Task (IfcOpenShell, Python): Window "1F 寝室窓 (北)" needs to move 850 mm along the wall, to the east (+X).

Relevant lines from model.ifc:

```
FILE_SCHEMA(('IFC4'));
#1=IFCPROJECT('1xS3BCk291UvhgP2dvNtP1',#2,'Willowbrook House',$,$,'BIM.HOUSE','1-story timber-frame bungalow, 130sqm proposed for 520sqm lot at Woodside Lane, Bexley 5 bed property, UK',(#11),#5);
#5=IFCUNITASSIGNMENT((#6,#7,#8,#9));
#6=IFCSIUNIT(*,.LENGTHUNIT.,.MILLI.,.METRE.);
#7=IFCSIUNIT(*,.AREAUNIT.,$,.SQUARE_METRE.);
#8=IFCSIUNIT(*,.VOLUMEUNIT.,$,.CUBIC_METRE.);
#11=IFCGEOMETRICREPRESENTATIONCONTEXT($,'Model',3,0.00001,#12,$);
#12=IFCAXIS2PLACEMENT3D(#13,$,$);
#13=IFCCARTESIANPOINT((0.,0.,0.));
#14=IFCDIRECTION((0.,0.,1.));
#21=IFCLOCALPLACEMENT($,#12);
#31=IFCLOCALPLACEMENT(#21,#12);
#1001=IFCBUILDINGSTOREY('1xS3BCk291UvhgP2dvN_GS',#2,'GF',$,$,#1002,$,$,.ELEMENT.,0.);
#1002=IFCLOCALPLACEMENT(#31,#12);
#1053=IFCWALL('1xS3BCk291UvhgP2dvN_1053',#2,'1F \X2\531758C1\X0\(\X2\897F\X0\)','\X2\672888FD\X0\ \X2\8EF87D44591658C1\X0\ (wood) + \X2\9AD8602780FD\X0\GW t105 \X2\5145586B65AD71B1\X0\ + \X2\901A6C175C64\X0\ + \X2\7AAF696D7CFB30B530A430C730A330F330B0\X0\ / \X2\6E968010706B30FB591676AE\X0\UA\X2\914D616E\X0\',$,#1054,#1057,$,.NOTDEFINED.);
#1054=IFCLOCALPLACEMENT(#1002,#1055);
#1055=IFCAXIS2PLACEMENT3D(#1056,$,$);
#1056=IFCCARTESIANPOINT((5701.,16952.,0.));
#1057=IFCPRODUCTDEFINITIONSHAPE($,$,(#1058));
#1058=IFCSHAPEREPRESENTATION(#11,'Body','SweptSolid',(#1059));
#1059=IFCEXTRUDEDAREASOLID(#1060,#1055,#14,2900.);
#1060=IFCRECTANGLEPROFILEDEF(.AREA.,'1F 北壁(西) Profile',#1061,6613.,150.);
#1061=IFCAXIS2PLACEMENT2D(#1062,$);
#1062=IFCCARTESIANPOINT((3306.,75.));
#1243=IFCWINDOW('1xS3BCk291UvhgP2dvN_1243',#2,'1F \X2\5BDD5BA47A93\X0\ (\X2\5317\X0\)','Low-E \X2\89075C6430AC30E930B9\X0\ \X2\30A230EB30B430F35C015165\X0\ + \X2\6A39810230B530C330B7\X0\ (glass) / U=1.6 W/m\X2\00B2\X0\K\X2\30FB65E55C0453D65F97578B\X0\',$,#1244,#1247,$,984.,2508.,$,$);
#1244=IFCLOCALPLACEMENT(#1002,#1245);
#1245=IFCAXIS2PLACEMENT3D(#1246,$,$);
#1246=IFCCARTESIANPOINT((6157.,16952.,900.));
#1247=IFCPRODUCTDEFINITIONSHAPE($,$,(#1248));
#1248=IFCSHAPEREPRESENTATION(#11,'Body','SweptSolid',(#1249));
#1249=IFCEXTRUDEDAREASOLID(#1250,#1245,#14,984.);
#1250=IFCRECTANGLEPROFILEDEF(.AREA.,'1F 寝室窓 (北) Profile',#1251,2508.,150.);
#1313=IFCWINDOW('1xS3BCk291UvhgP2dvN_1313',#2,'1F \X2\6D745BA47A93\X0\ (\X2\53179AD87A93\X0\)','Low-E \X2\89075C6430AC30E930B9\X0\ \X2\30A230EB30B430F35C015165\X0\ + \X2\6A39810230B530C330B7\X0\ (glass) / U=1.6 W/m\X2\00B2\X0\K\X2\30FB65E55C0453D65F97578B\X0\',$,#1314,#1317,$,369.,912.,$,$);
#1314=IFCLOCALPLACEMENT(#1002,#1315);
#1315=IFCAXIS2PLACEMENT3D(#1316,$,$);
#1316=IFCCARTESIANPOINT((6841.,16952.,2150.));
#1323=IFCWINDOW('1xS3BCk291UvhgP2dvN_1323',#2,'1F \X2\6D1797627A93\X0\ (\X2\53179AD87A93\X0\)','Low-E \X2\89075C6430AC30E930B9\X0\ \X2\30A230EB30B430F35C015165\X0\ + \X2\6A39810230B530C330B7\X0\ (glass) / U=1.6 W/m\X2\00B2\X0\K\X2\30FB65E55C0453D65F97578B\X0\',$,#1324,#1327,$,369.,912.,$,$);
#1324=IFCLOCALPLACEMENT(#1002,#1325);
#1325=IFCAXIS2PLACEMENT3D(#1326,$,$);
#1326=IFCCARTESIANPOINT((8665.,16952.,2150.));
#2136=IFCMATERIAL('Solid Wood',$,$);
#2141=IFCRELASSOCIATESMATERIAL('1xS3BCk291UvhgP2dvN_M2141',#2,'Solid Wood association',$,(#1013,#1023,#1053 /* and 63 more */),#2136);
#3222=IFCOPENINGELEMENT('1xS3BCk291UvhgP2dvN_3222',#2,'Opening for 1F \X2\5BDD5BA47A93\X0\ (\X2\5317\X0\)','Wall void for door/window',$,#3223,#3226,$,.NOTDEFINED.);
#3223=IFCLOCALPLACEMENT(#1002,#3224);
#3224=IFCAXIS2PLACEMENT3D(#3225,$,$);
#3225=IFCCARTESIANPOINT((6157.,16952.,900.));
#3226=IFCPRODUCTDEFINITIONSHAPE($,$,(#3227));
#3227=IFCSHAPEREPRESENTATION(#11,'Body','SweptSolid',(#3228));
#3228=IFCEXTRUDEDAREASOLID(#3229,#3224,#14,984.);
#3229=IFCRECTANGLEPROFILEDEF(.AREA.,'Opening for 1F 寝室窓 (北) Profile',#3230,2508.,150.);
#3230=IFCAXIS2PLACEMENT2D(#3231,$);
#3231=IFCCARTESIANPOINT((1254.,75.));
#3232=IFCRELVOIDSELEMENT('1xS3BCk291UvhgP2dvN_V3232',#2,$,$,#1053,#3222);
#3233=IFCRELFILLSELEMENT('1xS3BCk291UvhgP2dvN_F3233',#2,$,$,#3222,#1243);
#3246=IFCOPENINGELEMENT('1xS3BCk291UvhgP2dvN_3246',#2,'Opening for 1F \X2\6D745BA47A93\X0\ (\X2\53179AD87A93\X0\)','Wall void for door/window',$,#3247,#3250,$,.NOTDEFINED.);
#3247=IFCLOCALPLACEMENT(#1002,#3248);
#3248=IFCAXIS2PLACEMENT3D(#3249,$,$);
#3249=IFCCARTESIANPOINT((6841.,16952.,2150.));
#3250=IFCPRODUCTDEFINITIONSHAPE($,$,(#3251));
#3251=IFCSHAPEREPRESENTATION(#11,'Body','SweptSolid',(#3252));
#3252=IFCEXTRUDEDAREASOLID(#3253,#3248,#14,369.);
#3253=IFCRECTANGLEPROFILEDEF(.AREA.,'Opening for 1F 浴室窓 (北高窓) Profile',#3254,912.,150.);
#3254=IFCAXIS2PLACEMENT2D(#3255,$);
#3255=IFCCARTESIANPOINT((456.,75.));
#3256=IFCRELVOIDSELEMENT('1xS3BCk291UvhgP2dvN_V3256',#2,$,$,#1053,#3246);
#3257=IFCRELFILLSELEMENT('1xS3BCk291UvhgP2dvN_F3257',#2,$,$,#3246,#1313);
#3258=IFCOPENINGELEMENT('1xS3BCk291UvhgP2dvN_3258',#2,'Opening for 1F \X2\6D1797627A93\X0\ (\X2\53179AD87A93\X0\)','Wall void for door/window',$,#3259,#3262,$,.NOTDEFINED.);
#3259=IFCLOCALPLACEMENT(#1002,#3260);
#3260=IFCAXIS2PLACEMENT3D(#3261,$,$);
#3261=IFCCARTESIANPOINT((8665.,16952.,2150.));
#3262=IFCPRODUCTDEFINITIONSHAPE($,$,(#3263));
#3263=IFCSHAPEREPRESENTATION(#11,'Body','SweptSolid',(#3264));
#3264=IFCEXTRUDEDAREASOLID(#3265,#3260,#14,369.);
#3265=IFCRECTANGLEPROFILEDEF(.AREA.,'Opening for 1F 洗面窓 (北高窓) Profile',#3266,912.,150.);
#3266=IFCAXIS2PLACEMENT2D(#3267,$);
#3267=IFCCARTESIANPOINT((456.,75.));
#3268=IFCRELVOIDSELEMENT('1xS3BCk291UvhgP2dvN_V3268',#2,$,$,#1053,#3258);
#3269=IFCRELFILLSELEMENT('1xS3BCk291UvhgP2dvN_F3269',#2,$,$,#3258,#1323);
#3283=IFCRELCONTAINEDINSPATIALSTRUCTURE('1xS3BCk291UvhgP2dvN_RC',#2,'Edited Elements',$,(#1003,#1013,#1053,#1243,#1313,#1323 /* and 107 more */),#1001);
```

```python
import ifcopenshell
import ifcopenshell.api.geometry
import ifcopenshell.util.placement
import ifcopenshell.util.unit

model = ifcopenshell.open("model.ifc")
unit_scale = ifcopenshell.util.unit.calculate_unit_scale(model)

window = model.by_guid("1xS3BCk291UvhgP2dvN_1243")
opening = window.FillsVoids[0].RelatingOpeningElement
wall = opening.VoidsElements[0].RelatingBuildingElement

wall_matrix = ifcopenshell.util.placement.get_local_placement(wall.ObjectPlacement)
shift = wall_matrix[:3, 0] * 0.85 / unit_scale
before = ifcopenshell.util.placement.get_local_placement(window.ObjectPlacement)[:3, 3].copy()

# The window is not placed relative to its opening, so move both.
for product in (opening, window):
    matrix = ifcopenshell.util.placement.get_local_placement(product.ObjectPlacement)
    matrix[:3, 3] += shift
    ifcopenshell.api.geometry.edit_object_placement(model, product=product, matrix=matrix, is_si=False)

after = ifcopenshell.util.placement.get_local_placement(window.ObjectPlacement)[:3, 3]
print("window moved by", (after - before).round(3) + 0.0)

model.write("model_v2.ifc")
```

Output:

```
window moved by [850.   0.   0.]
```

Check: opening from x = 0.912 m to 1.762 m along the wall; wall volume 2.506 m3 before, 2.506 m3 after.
